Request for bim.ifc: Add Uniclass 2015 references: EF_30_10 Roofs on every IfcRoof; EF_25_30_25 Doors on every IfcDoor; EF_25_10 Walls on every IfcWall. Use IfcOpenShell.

First a look at what the model holds.

```python
import ifcopenshell

model = ifcopenshell.open("bim.ifc")
print(model.schema)
print("classifications:", [c.Name for c in model.by_type("IfcClassification")])
for ifc_class in ("IfcDoor", "IfcRoof", "IfcStair", "IfcWall", "IfcWindow"):
    print(ifc_class, len(model.by_type(ifc_class)))
```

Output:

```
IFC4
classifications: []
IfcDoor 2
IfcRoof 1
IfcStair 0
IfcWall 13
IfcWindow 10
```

```python
import ifcopenshell
import ifcopenshell.api.classification

model = ifcopenshell.open("bim.ifc")

system = ifcopenshell.api.classification.add_classification(model, classification="Uniclass 2015")

codes = {
    "IfcRoof": ("EF_30_10", "Roofs"),
    "IfcDoor": ("EF_25_30_25", "Doors"),
    "IfcWall": ("EF_25_10", "Walls"),
}
for ifc_class, (code, name) in codes.items():
    products = model.by_type(ifc_class)
    ifcopenshell.api.classification.add_reference(
        model, products=products, classification=system, identification=code, name=name
    )
    print(code, len(products))

model.write("bim_v2.ifc")
```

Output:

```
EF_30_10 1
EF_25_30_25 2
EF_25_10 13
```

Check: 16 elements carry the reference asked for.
